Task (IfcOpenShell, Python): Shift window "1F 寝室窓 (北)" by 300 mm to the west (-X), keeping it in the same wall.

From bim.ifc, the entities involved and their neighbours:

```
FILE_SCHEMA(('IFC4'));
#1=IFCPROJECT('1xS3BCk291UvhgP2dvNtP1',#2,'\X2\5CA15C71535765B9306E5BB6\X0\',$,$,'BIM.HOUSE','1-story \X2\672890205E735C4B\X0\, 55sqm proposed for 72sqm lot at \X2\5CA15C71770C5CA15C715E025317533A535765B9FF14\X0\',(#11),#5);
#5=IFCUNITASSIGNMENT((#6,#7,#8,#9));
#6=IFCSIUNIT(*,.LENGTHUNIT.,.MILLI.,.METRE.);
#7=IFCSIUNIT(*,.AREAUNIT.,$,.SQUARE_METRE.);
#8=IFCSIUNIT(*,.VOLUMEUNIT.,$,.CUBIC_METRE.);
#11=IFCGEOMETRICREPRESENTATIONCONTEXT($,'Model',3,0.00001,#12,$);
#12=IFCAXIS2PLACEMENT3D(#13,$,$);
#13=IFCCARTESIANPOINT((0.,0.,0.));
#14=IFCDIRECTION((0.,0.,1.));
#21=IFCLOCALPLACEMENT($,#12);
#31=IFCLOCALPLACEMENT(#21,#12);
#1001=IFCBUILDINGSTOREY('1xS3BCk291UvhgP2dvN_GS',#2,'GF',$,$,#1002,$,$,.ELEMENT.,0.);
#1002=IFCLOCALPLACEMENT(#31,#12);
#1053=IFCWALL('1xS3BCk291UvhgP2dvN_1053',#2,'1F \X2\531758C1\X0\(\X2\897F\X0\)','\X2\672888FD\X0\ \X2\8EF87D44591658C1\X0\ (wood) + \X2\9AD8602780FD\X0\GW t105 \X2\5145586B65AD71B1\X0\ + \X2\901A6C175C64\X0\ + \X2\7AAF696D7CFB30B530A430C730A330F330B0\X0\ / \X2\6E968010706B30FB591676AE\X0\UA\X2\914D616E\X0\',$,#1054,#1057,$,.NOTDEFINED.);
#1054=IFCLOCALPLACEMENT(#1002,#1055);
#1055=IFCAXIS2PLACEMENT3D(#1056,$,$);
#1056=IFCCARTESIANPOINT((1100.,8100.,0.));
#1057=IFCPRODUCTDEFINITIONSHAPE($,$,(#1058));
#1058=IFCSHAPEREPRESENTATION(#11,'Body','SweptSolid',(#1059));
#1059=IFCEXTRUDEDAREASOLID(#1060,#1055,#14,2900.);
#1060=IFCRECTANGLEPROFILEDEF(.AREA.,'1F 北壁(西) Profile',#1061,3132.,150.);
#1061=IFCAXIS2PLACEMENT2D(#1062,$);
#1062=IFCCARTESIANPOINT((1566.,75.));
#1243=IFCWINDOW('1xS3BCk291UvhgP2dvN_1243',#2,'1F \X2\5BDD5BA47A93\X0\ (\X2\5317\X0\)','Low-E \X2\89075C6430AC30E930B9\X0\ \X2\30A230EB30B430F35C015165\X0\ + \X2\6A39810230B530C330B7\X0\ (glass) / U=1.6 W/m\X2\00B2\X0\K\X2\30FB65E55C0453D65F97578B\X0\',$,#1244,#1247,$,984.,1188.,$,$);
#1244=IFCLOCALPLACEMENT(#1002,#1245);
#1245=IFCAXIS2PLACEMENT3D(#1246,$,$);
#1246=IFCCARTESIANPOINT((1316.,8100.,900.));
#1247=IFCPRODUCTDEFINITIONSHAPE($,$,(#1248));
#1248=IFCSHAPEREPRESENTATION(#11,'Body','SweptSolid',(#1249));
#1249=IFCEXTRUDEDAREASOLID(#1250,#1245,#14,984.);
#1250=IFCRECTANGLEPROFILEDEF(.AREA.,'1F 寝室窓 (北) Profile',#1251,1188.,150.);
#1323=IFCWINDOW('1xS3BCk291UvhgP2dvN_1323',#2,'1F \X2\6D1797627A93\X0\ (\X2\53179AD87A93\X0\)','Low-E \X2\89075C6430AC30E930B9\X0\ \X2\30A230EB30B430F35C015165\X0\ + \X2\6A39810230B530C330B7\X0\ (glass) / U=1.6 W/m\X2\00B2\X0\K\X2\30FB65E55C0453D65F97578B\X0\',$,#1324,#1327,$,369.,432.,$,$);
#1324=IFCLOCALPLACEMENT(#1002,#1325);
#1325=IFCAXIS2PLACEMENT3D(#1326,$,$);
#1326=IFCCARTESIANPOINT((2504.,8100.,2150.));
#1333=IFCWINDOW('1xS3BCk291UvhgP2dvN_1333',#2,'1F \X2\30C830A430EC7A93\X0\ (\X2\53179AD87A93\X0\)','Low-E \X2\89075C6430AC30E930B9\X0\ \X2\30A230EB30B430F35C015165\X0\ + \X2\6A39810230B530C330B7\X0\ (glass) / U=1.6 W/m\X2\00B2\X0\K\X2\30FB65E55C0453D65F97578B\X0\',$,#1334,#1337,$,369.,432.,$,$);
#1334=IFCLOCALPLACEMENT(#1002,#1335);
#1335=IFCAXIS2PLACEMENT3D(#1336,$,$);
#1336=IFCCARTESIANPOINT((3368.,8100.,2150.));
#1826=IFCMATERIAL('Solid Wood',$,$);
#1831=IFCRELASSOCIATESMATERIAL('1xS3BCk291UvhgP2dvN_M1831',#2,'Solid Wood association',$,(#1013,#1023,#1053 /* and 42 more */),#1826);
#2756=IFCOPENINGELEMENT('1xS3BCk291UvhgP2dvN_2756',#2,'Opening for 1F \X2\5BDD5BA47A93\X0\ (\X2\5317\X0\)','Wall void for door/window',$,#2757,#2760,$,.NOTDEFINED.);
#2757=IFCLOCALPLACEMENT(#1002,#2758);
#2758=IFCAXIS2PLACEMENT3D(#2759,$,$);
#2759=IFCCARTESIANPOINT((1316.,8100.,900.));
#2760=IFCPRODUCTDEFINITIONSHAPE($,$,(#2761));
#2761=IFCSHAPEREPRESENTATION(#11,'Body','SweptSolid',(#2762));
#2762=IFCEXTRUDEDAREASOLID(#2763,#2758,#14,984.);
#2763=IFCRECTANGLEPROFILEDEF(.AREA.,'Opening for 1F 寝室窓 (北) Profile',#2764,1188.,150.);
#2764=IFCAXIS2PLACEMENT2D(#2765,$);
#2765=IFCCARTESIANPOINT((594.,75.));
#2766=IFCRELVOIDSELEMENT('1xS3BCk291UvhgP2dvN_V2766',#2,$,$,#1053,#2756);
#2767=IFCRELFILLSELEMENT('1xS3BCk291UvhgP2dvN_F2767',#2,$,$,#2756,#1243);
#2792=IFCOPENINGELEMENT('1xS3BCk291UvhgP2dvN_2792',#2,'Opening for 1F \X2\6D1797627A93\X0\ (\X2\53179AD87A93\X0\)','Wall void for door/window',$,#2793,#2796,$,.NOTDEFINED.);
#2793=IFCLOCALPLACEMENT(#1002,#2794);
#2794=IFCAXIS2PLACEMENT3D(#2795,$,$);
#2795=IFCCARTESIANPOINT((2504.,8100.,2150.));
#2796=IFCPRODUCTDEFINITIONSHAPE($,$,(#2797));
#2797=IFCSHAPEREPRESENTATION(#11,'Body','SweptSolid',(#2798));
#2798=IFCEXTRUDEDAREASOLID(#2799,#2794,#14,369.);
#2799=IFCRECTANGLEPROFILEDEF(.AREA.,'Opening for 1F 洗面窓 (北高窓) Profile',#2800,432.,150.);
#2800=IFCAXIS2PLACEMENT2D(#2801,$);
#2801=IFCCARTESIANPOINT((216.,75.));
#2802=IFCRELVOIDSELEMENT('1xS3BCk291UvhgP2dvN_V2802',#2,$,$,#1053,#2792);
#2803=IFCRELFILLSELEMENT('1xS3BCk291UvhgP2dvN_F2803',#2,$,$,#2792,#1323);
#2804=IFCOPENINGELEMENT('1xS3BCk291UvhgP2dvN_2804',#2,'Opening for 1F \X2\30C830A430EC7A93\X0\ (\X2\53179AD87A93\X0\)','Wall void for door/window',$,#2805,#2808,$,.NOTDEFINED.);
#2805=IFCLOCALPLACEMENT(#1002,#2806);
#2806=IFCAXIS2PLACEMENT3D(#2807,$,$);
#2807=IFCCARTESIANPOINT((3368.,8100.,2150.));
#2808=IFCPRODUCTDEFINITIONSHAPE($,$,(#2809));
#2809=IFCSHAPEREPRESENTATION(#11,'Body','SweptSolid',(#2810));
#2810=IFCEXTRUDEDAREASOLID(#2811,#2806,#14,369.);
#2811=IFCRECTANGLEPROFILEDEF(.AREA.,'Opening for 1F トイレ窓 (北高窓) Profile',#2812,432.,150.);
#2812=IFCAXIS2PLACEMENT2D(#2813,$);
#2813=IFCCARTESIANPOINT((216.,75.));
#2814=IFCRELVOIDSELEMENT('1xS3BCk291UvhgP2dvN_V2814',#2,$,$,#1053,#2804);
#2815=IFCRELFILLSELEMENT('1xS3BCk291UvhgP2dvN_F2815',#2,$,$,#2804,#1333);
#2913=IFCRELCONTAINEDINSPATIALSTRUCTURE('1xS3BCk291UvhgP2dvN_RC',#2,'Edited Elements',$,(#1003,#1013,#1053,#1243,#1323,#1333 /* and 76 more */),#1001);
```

```python
import ifcopenshell
import ifcopenshell.api.geometry
import ifcopenshell.util.placement
import ifcopenshell.util.unit

model = ifcopenshell.open("bim.ifc")
unit_scale = ifcopenshell.util.unit.calculate_unit_scale(model)

window = model.by_guid("1xS3BCk291UvhgP2dvN_1243")
opening = window.FillsVoids[0].RelatingOpeningElement
wall = opening.VoidsElements[0].RelatingBuildingElement

wall_matrix = ifcopenshell.util.placement.get_local_placement(wall.ObjectPlacement)
shift = wall_matrix[:3, 0] * -0.3 / unit_scale
before = ifcopenshell.util.placement.get_local_placement(window.ObjectPlacement)[:3, 3].copy()

# The window is not placed relative to its opening, so move both.
for product in (opening, window):
    matrix = ifcopenshell.util.placement.get_local_placement(product.ObjectPlacement)
    matrix[:3, 3] += shift
    ifcopenshell.api.geometry.edit_object_placement(model, product=product, matrix=matrix, is_si=False)

after = ifcopenshell.util.placement.get_local_placement(window.ObjectPlacement)[:3, 3]
print("window moved by", (after - before).round(3) + 0.0)

model.write("bim-out.ifc")
```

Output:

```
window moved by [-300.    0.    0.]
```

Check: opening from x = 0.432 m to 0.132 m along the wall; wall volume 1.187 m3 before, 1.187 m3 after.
